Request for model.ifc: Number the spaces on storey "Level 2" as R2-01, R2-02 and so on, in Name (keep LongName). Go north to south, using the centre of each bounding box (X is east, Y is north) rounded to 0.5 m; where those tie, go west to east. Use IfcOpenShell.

First a look at what the model holds.

```python
import ifcopenshell
import ifcopenshell.util.element
import ifcopenshell.util.placement

model = ifcopenshell.open("model.ifc")
print(model.schema)
storey = next(s for s in model.by_type("IfcBuildingStorey") if s.Name == "Level 2")
spaces = [e for e in ifcopenshell.util.element.get_decomposition(storey) if e.is_a("IfcSpace")]
for e in sorted(spaces, key=lambda e: e.id()):
    origin = ifcopenshell.util.placement.get_local_placement(e.ObjectPlacement)[:3, 3]
    print(e.id(), e.Name, e.LongName, origin.round(2) + 0.0, sep=" | ")
```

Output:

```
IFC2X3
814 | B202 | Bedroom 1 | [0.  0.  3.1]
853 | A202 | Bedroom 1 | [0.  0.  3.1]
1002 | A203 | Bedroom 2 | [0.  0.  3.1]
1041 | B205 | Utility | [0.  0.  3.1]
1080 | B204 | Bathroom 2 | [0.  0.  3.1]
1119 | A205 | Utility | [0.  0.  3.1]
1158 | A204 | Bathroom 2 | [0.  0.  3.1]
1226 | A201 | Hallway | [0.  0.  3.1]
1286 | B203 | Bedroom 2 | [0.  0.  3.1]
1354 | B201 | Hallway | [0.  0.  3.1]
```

```python
import ifcopenshell
import ifcopenshell.geom
import ifcopenshell.util.element
import ifcopenshell.util.shape

model = ifcopenshell.open("model.ifc")
settings = ifcopenshell.geom.settings()
settings.set("use-world-coords", True)


def centre(element):
    shape = ifcopenshell.geom.create_shape(settings, element)
    return ifcopenshell.util.shape.get_bbox_centroid(shape.geometry)


storey = next(s for s in model.by_type("IfcBuildingStorey") if s.Name == "Level 2")
spaces = [e for e in ifcopenshell.util.element.get_decomposition(storey) if e.is_a("IfcSpace")]

# Insertion points can sit at a corner or the storey origin, so sort by the geometry (in metres).
centres = {e: centre(e) for e in spaces}
spaces.sort(key=lambda e: (-round(centres[e][1] / 0.5), centres[e][0]))

for i, e in enumerate(spaces, start=1):
    number = f"R2-{i:02d}"
    e.Name = number
    print(e.id(), number)

model.write("model_updated.ifc")
```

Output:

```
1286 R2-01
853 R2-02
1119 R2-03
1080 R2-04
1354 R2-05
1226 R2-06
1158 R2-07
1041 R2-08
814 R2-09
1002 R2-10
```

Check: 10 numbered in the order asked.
